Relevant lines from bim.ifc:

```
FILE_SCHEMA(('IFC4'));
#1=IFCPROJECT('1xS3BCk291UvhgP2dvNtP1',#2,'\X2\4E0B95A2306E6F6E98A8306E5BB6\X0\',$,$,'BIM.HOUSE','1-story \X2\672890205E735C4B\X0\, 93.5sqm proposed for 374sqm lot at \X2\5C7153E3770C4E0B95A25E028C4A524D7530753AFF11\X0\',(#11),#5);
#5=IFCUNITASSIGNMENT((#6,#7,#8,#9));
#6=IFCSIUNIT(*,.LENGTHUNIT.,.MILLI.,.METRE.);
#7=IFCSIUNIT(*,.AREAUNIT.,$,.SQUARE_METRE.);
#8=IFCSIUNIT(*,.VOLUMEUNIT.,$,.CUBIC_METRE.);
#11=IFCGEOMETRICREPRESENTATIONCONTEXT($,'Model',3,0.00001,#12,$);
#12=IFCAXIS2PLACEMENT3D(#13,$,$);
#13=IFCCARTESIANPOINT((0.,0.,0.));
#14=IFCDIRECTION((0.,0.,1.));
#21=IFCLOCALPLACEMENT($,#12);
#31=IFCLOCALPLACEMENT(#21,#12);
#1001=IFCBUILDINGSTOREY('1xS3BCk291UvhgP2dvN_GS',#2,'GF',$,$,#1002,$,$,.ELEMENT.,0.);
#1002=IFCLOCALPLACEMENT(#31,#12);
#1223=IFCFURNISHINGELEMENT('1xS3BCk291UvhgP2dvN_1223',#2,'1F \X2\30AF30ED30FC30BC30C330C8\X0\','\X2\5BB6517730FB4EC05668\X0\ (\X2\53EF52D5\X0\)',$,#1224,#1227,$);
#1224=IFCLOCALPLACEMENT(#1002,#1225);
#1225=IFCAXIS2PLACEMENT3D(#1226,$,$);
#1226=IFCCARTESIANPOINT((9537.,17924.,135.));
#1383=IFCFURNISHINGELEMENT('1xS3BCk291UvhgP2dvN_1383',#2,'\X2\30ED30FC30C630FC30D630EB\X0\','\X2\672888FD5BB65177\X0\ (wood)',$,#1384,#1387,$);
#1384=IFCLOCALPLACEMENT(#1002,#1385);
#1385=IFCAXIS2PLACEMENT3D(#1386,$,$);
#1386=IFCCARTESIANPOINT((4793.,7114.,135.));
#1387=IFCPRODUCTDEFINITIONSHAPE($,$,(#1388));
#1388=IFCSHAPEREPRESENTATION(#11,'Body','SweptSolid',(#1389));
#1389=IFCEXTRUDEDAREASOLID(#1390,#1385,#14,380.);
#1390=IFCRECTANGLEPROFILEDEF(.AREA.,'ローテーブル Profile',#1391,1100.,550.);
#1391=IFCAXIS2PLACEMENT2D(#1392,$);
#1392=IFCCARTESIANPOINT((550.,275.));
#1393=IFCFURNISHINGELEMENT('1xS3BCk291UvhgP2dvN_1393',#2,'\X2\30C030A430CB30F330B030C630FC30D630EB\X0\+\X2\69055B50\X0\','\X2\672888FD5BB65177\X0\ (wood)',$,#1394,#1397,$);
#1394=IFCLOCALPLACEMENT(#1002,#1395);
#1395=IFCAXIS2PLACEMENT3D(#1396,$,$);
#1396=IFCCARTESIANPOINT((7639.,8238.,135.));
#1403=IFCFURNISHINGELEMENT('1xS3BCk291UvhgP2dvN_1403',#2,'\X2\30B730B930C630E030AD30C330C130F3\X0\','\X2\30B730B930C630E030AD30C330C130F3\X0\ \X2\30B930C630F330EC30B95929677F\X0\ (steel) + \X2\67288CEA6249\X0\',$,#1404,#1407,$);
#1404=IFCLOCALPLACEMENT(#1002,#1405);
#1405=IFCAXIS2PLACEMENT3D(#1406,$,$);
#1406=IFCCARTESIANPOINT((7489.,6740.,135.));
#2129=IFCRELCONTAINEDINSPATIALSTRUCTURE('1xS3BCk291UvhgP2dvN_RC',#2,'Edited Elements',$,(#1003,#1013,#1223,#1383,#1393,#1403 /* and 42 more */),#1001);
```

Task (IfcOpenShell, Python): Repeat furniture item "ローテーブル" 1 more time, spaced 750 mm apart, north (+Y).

```python
import numpy as np
import ifcopenshell
import ifcopenshell.api.geometry
import ifcopenshell.api.root
import ifcopenshell.util.element
import ifcopenshell.util.placement

model = ifcopenshell.open("bim.ifc")


def reuse_history(source, copy):
    """copy_class also copies each property set's owner history, people and application; keep the originals."""
    for rel in copy.IsDefinedBy:
        if rel.is_a("IfcRelDefinesByProperties") and (history := rel.RelatingPropertyDefinition.OwnerHistory):
            rel.RelatingPropertyDefinition.OwnerHistory = source.OwnerHistory
            ifcopenshell.util.element.remove_deep2(model, history)


source = model.by_id(1383)
base = ifcopenshell.util.placement.get_local_placement(source.ObjectPlacement)
step = np.array([0.0, 1.0, 0.0]) * 750.0

for i in range(1, 2):
    copy = ifcopenshell.api.root.copy_class(model, product=source)
    copy.Representation = ifcopenshell.util.element.copy_deep(
        model, source.Representation, exclude=["IfcGeometricRepresentationContext", "IfcRepresentationMap"]
    )
    reuse_history(source, copy)
    matrix = base.copy()
    matrix[:3, 3] += i * step
    print("added at", matrix[:3, 3].round(3) + 0.0)
    ifcopenshell.api.geometry.edit_object_placement(model, product=copy, matrix=matrix, is_si=False)

model.write("bim_v2.ifc")
```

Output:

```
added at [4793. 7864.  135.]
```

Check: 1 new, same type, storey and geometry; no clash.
